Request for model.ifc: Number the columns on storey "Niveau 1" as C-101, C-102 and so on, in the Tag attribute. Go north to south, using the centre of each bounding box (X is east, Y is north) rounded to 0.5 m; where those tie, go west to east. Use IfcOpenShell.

First a look at what the model holds.

```python
import ifcopenshell
import ifcopenshell.util.element
import ifcopenshell.util.placement

model = ifcopenshell.open("model.ifc")
print(model.schema)
storey = next(s for s in model.by_type("IfcBuildingStorey") if s.Name == "Niveau 1")
columns = [e for e in ifcopenshell.util.element.get_decomposition(storey) if e.is_a("IfcColumn")]
for e in sorted(columns, key=lambda e: e.id()):
    origin = ifcopenshell.util.placement.get_local_placement(e.ObjectPlacement)[:3, 3]
    print(e.id(), e.Tag, e.Name, origin.round(2) + 0.0, sep=" | ")
```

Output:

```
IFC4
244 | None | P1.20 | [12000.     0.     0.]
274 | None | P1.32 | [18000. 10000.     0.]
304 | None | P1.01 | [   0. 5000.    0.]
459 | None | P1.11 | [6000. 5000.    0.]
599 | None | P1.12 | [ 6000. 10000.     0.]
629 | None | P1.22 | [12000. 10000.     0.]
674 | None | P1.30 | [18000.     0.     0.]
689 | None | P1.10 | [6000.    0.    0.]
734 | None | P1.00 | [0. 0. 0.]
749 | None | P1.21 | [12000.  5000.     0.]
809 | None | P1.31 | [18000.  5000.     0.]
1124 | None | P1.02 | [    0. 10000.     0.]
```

```python
import ifcopenshell
import ifcopenshell.geom
import ifcopenshell.util.element
import ifcopenshell.util.shape

model = ifcopenshell.open("model.ifc")
settings = ifcopenshell.geom.settings()
settings.set("use-world-coords", True)


def centre(element):
    shape = ifcopenshell.geom.create_shape(settings, element)
    return ifcopenshell.util.shape.get_bbox_centroid(shape.geometry)


storey = next(s for s in model.by_type("IfcBuildingStorey") if s.Name == "Niveau 1")
columns = [e for e in ifcopenshell.util.element.get_decomposition(storey) if e.is_a("IfcColumn")]

# Insertion points can sit at a corner or the storey origin, so sort by the geometry (in metres).
centres = {e: centre(e) for e in columns}
columns.sort(key=lambda e: (-round(centres[e][1] / 0.5), centres[e][0]))

for i, e in enumerate(columns, start=1):
    number = f"C-1{i:02d}"
    e.Tag = number
    print(e.id(), number)

model.write("model_v2.ifc")
```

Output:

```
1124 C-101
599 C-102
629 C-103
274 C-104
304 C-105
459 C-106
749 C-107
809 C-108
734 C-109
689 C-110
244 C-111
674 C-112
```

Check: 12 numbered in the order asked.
